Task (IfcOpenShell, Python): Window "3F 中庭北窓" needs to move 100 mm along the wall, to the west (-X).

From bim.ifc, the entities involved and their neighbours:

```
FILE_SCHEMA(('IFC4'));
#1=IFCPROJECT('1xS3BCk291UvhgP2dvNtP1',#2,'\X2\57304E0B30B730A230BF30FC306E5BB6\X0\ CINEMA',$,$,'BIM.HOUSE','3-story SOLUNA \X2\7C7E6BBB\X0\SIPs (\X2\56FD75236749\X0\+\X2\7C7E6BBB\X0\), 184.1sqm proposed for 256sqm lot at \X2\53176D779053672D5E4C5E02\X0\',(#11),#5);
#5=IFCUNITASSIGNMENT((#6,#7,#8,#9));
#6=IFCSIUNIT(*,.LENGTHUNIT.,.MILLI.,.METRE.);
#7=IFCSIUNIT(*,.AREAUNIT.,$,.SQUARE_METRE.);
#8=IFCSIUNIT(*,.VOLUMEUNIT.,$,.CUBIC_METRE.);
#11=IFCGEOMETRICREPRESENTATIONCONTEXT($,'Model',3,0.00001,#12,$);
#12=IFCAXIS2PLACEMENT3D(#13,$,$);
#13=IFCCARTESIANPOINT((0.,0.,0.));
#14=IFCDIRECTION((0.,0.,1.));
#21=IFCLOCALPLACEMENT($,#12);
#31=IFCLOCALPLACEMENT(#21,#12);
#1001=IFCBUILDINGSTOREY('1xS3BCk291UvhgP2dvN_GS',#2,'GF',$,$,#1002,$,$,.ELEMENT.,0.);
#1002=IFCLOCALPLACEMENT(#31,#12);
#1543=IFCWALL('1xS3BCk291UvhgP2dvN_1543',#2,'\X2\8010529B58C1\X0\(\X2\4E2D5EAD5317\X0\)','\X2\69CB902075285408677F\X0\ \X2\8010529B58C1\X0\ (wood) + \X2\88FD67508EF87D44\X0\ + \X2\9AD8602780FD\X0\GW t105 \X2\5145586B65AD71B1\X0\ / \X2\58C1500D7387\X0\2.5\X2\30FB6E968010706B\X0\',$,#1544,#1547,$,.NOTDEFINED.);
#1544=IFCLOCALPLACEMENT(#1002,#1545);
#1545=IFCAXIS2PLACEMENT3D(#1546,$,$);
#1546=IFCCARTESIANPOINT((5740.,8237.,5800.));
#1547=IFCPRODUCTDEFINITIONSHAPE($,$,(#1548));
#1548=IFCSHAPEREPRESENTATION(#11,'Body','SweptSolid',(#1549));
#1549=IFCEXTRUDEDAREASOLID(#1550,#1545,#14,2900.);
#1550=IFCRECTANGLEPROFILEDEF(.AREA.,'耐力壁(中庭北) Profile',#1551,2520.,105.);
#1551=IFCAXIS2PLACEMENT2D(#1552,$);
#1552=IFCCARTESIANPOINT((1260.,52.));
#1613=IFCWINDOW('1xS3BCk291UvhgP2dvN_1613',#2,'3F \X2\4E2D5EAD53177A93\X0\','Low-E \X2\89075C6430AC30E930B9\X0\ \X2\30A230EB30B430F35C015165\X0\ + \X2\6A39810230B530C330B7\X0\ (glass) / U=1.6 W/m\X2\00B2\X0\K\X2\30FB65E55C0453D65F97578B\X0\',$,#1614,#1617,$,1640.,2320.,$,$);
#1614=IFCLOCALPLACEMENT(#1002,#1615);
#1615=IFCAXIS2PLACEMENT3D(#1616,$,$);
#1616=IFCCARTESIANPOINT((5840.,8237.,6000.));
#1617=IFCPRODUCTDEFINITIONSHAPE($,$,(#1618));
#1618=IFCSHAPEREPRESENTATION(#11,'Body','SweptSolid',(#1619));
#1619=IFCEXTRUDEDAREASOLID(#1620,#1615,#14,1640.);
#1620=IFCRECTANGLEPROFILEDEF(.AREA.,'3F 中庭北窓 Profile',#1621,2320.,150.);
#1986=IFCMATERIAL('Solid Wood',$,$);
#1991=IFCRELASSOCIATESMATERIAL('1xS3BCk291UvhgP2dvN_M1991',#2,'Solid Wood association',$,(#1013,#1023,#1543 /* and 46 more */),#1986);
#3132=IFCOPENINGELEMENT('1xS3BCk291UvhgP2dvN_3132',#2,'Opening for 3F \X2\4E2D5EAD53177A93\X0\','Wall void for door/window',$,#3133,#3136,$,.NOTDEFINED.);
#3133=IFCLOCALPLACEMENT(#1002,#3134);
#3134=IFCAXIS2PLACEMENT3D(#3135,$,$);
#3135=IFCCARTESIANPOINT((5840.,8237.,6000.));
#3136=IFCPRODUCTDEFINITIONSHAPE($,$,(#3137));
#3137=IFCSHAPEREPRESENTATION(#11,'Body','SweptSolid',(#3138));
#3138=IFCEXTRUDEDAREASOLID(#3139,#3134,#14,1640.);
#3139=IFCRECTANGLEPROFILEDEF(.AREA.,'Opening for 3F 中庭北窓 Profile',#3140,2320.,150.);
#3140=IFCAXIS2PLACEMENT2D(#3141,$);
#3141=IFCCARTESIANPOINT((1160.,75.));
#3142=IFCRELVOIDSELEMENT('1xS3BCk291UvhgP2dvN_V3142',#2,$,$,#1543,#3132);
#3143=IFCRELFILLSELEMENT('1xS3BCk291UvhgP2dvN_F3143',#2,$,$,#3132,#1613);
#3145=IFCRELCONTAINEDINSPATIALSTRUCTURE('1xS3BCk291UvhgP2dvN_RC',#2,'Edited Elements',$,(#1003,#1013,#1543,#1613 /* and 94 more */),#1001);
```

```python
import ifcopenshell
import ifcopenshell.api.geometry
import ifcopenshell.util.placement
import ifcopenshell.util.unit

model = ifcopenshell.open("bim.ifc")
unit_scale = ifcopenshell.util.unit.calculate_unit_scale(model)

window = model.by_id(1613)
opening = window.FillsVoids[0].RelatingOpeningElement
wall = opening.VoidsElements[0].RelatingBuildingElement

wall_matrix = ifcopenshell.util.placement.get_local_placement(wall.ObjectPlacement)
shift = wall_matrix[:3, 0] * -0.1 / unit_scale
before = ifcopenshell.util.placement.get_local_placement(window.ObjectPlacement)[:3, 3].copy()

# The window is not placed relative to its opening, so move both.
for product in (opening, window):
    matrix = ifcopenshell.util.placement.get_local_placement(product.ObjectPlacement)
    matrix[:3, 3] += shift
    ifcopenshell.api.geometry.edit_object_placement(model, product=product, matrix=matrix, is_si=False)

after = ifcopenshell.util.placement.get_local_placement(window.ObjectPlacement)[:3, 3]
print("window moved by", (after - before).round(3) + 0.0)

model.write("bim_v2.ifc")
```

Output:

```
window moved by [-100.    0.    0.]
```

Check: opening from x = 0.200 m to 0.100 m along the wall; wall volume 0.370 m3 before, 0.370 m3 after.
